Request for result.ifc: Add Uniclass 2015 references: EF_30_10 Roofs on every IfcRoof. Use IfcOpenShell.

First a look at what the model holds.

```python
import ifcopenshell

model = ifcopenshell.open("result.ifc")
print(model.schema)
print("classifications:", [c.Name for c in model.by_type("IfcClassification")])
for ifc_class in ("IfcDoor", "IfcRoof", "IfcStair", "IfcWall", "IfcWindow"):
    print(ifc_class, len(model.by_type(ifc_class)))
```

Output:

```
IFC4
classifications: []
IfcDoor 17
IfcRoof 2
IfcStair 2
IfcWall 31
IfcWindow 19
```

```python
import ifcopenshell
import ifcopenshell.api.classification

model = ifcopenshell.open("result.ifc")

system = ifcopenshell.api.classification.add_classification(model, classification="Uniclass 2015")

codes = {
    "IfcRoof": ("EF_30_10", "Roofs"),
}
for ifc_class, (code, name) in codes.items():
    products = model.by_type(ifc_class)
    ifcopenshell.api.classification.add_reference(
        model, products=products, classification=system, identification=code, name=name
    )
    print(code, len(products))

model.write("result_rev.ifc")
```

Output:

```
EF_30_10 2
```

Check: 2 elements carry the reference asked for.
